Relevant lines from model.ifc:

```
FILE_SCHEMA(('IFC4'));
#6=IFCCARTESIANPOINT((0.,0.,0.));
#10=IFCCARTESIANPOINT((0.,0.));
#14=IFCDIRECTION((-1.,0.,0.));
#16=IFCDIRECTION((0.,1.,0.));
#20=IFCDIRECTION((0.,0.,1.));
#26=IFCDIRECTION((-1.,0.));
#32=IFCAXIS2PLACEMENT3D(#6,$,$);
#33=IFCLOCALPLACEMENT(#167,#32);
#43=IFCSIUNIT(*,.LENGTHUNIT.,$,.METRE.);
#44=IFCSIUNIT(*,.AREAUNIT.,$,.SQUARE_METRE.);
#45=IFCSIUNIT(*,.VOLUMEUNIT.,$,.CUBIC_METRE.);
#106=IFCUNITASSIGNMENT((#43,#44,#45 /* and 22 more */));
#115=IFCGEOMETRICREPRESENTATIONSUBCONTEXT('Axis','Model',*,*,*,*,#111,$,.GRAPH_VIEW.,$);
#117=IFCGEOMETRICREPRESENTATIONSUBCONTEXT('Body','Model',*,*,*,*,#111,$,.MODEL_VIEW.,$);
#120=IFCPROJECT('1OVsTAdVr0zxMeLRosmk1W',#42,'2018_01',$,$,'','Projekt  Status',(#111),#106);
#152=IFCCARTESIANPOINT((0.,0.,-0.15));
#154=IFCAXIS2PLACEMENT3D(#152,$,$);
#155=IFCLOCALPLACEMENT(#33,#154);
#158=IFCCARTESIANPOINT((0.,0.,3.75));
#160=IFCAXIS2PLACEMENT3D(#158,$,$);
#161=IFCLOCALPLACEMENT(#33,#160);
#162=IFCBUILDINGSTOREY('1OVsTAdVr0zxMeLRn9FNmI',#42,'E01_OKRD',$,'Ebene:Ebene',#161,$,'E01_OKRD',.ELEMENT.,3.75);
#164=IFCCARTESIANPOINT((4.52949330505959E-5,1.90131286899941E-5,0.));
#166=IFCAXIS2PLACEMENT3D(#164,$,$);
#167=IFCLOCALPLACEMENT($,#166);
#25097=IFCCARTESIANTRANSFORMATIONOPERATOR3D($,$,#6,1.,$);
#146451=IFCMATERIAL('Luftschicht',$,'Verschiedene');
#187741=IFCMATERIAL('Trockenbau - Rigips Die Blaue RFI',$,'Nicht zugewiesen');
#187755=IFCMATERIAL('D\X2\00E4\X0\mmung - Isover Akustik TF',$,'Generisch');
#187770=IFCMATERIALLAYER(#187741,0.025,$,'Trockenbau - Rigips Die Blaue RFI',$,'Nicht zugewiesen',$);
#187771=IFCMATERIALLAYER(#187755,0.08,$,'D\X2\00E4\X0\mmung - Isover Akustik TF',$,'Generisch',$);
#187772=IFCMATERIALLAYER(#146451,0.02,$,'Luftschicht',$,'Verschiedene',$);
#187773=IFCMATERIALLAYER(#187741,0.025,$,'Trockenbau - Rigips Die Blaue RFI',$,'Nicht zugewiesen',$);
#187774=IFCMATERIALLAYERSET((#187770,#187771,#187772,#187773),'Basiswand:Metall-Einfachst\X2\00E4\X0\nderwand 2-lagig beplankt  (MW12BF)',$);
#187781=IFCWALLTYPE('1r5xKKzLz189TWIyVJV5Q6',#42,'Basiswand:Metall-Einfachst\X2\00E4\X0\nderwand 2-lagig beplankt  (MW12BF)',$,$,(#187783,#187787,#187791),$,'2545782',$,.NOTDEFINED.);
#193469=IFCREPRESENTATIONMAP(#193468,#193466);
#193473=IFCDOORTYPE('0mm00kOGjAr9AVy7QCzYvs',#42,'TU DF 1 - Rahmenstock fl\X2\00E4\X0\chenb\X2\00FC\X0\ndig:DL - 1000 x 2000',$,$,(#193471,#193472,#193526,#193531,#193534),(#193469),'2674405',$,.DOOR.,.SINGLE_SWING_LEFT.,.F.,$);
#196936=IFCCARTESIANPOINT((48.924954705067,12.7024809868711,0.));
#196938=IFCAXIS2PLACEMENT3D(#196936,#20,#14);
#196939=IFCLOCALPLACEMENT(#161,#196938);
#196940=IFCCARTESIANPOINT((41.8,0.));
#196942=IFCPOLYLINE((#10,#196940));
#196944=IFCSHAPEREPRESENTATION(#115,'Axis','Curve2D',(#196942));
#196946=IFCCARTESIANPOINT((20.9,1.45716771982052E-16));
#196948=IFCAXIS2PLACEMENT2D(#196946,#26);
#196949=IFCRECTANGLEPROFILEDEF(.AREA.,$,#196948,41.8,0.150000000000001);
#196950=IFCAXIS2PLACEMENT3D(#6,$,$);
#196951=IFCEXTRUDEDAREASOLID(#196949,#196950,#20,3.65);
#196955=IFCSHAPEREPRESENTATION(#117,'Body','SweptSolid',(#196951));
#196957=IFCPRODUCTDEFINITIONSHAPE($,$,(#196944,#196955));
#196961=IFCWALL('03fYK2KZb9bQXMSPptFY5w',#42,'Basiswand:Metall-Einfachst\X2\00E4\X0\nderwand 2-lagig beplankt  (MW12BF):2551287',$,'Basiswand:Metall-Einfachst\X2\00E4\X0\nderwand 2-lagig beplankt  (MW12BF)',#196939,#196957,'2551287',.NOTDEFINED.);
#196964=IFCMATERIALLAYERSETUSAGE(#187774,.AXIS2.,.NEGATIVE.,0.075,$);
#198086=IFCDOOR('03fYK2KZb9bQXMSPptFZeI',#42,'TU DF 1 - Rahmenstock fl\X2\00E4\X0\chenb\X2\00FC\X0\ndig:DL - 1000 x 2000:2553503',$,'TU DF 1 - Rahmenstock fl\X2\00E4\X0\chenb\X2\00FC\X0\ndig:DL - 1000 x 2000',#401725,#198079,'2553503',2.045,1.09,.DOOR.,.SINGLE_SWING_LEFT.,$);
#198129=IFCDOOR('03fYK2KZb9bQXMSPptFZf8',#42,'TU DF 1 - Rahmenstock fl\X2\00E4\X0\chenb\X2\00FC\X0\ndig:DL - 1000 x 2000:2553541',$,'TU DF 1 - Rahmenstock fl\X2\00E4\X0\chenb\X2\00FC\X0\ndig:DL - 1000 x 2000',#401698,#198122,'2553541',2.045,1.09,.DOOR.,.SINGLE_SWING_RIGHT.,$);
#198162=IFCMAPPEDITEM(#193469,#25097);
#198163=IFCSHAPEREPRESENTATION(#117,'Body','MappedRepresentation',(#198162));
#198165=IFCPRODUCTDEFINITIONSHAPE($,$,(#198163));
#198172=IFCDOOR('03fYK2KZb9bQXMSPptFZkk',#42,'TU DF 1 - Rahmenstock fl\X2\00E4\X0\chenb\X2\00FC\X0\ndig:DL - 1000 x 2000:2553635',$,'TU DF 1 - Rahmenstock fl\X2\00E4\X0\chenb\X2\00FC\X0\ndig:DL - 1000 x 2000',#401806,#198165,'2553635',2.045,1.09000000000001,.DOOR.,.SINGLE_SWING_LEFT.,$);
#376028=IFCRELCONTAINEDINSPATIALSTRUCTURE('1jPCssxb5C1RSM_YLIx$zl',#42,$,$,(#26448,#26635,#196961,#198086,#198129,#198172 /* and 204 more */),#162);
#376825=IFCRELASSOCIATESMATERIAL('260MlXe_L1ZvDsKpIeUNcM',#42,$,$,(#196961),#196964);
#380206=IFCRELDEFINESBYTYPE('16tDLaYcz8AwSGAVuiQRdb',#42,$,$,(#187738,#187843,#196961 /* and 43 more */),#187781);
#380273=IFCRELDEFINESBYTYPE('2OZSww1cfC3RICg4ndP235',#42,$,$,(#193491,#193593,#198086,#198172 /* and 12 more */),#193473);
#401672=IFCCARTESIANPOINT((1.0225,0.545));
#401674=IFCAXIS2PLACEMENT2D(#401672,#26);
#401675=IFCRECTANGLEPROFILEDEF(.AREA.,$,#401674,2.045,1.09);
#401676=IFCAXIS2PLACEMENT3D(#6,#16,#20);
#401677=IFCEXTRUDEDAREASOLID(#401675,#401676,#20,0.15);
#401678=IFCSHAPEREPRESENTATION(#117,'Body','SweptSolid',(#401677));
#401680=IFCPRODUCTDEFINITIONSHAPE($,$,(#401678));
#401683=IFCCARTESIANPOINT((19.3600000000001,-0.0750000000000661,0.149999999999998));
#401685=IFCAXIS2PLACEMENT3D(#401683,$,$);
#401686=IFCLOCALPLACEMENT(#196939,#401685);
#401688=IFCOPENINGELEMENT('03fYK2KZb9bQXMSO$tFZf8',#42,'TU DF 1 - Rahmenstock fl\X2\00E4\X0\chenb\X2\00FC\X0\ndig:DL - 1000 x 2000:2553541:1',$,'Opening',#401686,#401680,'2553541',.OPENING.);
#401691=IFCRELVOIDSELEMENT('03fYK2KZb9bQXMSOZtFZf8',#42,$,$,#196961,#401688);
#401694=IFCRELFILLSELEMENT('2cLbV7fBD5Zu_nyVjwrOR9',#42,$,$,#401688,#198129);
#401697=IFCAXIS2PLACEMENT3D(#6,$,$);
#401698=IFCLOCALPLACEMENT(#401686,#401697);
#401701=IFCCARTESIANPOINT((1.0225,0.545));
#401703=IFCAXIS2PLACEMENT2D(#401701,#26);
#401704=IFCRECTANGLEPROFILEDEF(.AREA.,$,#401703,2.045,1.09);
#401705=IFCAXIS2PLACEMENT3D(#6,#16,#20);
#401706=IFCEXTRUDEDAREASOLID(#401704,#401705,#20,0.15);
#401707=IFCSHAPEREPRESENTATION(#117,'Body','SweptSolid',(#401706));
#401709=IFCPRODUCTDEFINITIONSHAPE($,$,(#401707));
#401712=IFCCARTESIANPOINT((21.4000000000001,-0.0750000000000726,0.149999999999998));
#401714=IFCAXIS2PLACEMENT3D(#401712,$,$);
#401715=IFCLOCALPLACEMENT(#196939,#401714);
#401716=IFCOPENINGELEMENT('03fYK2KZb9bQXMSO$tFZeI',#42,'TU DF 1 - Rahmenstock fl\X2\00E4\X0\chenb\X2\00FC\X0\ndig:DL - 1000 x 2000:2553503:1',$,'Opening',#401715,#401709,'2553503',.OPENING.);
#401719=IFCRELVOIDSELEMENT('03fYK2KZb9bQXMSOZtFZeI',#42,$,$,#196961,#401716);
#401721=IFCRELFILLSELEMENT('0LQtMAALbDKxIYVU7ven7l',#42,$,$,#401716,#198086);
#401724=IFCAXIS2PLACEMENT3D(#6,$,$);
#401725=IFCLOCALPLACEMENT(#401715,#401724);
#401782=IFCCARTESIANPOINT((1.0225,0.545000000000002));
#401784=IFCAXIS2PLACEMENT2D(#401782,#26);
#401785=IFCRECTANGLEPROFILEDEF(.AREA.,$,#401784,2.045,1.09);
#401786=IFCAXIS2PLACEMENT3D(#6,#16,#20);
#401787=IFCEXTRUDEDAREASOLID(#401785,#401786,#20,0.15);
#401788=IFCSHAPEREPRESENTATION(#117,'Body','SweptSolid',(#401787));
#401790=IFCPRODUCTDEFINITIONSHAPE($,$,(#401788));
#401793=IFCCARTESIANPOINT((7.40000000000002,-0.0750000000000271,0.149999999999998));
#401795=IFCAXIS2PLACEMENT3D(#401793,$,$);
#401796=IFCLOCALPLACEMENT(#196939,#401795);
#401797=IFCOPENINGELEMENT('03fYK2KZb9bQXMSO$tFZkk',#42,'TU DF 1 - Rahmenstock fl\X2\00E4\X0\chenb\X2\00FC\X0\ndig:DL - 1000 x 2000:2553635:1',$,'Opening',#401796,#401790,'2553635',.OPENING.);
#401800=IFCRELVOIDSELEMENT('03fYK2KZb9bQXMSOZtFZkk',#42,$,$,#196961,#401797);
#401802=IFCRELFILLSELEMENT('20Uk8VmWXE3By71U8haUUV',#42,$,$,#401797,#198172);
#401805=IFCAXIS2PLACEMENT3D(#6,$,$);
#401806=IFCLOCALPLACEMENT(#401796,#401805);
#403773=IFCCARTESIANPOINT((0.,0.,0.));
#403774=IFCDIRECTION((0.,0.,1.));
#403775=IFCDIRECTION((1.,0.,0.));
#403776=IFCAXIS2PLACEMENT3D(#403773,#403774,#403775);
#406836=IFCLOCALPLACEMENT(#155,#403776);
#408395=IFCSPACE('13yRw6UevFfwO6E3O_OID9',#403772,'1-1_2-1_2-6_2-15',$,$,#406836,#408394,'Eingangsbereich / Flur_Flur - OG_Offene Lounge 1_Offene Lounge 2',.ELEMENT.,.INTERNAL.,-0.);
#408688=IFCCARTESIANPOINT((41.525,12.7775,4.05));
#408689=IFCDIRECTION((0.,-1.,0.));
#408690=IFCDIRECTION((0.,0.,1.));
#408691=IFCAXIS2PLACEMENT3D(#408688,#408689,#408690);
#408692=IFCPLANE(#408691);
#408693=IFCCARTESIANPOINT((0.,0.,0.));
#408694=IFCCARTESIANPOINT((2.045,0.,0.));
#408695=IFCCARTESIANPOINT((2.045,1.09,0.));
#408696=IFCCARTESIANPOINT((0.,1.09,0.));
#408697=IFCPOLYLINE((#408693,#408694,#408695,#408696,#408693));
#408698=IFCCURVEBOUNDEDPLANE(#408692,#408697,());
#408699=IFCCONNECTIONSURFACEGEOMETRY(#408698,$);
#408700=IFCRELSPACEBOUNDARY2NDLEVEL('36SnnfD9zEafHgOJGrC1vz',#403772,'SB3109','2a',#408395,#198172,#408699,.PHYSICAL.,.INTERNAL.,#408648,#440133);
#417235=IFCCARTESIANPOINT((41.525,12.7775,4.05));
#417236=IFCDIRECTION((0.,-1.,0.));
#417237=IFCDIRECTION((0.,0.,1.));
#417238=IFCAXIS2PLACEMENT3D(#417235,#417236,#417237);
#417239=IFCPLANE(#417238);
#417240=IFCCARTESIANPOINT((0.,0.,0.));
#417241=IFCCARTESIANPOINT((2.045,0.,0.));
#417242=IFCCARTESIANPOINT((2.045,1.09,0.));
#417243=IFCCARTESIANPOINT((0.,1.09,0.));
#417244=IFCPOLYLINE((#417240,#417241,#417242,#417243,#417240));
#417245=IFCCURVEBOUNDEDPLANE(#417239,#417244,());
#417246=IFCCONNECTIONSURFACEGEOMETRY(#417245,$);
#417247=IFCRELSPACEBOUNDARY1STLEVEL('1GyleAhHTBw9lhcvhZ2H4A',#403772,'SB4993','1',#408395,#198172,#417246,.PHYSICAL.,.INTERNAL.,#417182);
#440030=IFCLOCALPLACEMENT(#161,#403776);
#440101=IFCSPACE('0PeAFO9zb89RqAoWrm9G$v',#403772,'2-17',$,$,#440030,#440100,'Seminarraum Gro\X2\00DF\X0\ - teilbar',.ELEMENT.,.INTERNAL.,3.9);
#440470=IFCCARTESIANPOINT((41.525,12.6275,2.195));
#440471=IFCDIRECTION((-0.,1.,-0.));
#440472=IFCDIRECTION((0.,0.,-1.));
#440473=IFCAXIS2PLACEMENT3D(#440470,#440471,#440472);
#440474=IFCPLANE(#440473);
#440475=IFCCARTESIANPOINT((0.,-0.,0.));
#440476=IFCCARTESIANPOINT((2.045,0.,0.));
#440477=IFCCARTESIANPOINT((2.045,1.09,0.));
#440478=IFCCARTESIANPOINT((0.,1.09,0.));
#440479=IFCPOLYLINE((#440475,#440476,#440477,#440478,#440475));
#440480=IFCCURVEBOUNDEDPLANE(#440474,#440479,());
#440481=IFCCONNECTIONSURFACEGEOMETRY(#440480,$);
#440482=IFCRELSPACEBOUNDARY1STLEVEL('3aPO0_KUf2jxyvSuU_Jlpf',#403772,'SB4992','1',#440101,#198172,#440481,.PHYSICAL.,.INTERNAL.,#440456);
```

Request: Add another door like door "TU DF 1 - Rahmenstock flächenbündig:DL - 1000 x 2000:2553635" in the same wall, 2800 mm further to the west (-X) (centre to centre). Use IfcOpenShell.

```python
import numpy as np
import ifcopenshell
import ifcopenshell.api.feature
import ifcopenshell.api.geometry
import ifcopenshell.api.root
import ifcopenshell.geom
import ifcopenshell.util.element
import ifcopenshell.util.placement
import ifcopenshell.util.shape
import ifcopenshell.util.unit

model = ifcopenshell.open("model.ifc")
unit_scale = ifcopenshell.util.unit.calculate_unit_scale(model)
settings = ifcopenshell.geom.settings()


def volume(element):
    """Net volume in cubic metres, openings subtracted."""
    shape = ifcopenshell.geom.create_shape(settings, element)
    return ifcopenshell.util.shape.get_volume(shape.geometry)


def reuse_history(source, copy):
    """copy_class also copies each property set's owner history, people and application; keep the originals."""
    for rel in copy.IsDefinedBy:
        if rel.is_a("IfcRelDefinesByProperties") and (history := rel.RelatingPropertyDefinition.OwnerHistory):
            rel.RelatingPropertyDefinition.OwnerHistory = source.OwnerHistory
            ifcopenshell.util.element.remove_deep2(model, history)


door = model.by_guid("03fYK2KZb9bQXMSPptFZkk")
opening = door.FillsVoids[0].RelatingOpeningElement
wall = opening.VoidsElements[0].RelatingBuildingElement
before = volume(wall)
shift = ifcopenshell.util.placement.get_local_placement(wall.ObjectPlacement)[:3, 0] * 2.8 / unit_scale

# copy_class copies the void relationship, type, container and properties, but no geometry.
new_opening = ifcopenshell.api.root.copy_class(model, product=opening)
new_opening.Representation = ifcopenshell.util.element.copy_deep(
    model, opening.Representation, exclude=["IfcGeometricRepresentationContext", "IfcRepresentationMap"]
)
new_opening.Name = "TU DF 1 - Rahmenstock flächenbündig:DL - 1000 x 2000"
new_opening.Tag = None
new_door = ifcopenshell.api.root.copy_class(model, product=door)
new_door.Representation = ifcopenshell.util.element.copy_deep(
    model, door.Representation, exclude=["IfcGeometricRepresentationContext", "IfcRepresentationMap"]
)
new_door.Name = "TU DF 1 - Rahmenstock flächenbündig:DL - 1000 x 2000"
new_door.Tag = None
reuse_history(door, new_door)
ifcopenshell.api.feature.add_filling(model, opening=new_opening, element=new_door)

for old, new in ((opening, new_opening), (door, new_door)):
    matrix = ifcopenshell.util.placement.get_local_placement(old.ObjectPlacement)
    matrix[:3, 3] += shift
    ifcopenshell.api.geometry.edit_object_placement(model, product=new, matrix=matrix, is_si=False)

# The copied space boundaries still share their surfaces with the original.
for rel in new_door.ProvidesBoundaries:
    if rel.ConnectionGeometry:
        rel.ConnectionGeometry = ifcopenshell.util.element.copy_deep(model, rel.ConnectionGeometry)

# Space boundary surfaces are stored in each space's coordinates; move them too.
for rel in new_door.ProvidesBoundaries:
    if not rel.ConnectionGeometry:
        continue
    surface = rel.ConnectionGeometry.SurfaceOnRelatingElement.BasisSurface
    space_matrix = ifcopenshell.util.placement.get_local_placement(rel.RelatingSpace.ObjectPlacement)
    point = np.array(surface.Position.Location.Coordinates) + space_matrix[:3, :3].T @ shift
    surface.Position = model.createIfcAxis2Placement3D(
        model.createIfcCartesianPoint(point.tolist()), surface.Position.Axis, surface.Position.RefDirection
    )

after = volume(wall)

print(f"wall volume {before:.3f} -> {after:.3f} m3")

model.write("model_v2.ifc")
```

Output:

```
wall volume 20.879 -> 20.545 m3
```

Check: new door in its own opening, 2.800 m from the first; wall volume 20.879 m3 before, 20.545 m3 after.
